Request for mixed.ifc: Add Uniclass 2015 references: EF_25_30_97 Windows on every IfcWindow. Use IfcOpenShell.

First a look at what the model holds.

```python
import ifcopenshell

model = ifcopenshell.open("mixed.ifc")
print(model.schema)
print("classifications:", [c.Name for c in model.by_type("IfcClassification")])
for ifc_class in ("IfcDoor", "IfcRoof", "IfcStair", "IfcWall", "IfcWindow"):
    print(ifc_class, len(model.by_type(ifc_class)))
```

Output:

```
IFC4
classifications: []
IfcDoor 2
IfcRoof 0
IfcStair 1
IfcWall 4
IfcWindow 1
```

```python
import ifcopenshell
import ifcopenshell.api.classification

model = ifcopenshell.open("mixed.ifc")

system = ifcopenshell.api.classification.add_classification(model, classification="Uniclass 2015")

codes = {
    "IfcWindow": ("EF_25_30_97", "Windows"),
}
for ifc_class, (code, name) in codes.items():
    products = model.by_type(ifc_class)
    ifcopenshell.api.classification.add_reference(
        model, products=products, classification=system, identification=code, name=name
    )
    print(code, len(products))

model.write("mixed_rev.ifc")
```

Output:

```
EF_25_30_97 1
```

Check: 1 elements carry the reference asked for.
